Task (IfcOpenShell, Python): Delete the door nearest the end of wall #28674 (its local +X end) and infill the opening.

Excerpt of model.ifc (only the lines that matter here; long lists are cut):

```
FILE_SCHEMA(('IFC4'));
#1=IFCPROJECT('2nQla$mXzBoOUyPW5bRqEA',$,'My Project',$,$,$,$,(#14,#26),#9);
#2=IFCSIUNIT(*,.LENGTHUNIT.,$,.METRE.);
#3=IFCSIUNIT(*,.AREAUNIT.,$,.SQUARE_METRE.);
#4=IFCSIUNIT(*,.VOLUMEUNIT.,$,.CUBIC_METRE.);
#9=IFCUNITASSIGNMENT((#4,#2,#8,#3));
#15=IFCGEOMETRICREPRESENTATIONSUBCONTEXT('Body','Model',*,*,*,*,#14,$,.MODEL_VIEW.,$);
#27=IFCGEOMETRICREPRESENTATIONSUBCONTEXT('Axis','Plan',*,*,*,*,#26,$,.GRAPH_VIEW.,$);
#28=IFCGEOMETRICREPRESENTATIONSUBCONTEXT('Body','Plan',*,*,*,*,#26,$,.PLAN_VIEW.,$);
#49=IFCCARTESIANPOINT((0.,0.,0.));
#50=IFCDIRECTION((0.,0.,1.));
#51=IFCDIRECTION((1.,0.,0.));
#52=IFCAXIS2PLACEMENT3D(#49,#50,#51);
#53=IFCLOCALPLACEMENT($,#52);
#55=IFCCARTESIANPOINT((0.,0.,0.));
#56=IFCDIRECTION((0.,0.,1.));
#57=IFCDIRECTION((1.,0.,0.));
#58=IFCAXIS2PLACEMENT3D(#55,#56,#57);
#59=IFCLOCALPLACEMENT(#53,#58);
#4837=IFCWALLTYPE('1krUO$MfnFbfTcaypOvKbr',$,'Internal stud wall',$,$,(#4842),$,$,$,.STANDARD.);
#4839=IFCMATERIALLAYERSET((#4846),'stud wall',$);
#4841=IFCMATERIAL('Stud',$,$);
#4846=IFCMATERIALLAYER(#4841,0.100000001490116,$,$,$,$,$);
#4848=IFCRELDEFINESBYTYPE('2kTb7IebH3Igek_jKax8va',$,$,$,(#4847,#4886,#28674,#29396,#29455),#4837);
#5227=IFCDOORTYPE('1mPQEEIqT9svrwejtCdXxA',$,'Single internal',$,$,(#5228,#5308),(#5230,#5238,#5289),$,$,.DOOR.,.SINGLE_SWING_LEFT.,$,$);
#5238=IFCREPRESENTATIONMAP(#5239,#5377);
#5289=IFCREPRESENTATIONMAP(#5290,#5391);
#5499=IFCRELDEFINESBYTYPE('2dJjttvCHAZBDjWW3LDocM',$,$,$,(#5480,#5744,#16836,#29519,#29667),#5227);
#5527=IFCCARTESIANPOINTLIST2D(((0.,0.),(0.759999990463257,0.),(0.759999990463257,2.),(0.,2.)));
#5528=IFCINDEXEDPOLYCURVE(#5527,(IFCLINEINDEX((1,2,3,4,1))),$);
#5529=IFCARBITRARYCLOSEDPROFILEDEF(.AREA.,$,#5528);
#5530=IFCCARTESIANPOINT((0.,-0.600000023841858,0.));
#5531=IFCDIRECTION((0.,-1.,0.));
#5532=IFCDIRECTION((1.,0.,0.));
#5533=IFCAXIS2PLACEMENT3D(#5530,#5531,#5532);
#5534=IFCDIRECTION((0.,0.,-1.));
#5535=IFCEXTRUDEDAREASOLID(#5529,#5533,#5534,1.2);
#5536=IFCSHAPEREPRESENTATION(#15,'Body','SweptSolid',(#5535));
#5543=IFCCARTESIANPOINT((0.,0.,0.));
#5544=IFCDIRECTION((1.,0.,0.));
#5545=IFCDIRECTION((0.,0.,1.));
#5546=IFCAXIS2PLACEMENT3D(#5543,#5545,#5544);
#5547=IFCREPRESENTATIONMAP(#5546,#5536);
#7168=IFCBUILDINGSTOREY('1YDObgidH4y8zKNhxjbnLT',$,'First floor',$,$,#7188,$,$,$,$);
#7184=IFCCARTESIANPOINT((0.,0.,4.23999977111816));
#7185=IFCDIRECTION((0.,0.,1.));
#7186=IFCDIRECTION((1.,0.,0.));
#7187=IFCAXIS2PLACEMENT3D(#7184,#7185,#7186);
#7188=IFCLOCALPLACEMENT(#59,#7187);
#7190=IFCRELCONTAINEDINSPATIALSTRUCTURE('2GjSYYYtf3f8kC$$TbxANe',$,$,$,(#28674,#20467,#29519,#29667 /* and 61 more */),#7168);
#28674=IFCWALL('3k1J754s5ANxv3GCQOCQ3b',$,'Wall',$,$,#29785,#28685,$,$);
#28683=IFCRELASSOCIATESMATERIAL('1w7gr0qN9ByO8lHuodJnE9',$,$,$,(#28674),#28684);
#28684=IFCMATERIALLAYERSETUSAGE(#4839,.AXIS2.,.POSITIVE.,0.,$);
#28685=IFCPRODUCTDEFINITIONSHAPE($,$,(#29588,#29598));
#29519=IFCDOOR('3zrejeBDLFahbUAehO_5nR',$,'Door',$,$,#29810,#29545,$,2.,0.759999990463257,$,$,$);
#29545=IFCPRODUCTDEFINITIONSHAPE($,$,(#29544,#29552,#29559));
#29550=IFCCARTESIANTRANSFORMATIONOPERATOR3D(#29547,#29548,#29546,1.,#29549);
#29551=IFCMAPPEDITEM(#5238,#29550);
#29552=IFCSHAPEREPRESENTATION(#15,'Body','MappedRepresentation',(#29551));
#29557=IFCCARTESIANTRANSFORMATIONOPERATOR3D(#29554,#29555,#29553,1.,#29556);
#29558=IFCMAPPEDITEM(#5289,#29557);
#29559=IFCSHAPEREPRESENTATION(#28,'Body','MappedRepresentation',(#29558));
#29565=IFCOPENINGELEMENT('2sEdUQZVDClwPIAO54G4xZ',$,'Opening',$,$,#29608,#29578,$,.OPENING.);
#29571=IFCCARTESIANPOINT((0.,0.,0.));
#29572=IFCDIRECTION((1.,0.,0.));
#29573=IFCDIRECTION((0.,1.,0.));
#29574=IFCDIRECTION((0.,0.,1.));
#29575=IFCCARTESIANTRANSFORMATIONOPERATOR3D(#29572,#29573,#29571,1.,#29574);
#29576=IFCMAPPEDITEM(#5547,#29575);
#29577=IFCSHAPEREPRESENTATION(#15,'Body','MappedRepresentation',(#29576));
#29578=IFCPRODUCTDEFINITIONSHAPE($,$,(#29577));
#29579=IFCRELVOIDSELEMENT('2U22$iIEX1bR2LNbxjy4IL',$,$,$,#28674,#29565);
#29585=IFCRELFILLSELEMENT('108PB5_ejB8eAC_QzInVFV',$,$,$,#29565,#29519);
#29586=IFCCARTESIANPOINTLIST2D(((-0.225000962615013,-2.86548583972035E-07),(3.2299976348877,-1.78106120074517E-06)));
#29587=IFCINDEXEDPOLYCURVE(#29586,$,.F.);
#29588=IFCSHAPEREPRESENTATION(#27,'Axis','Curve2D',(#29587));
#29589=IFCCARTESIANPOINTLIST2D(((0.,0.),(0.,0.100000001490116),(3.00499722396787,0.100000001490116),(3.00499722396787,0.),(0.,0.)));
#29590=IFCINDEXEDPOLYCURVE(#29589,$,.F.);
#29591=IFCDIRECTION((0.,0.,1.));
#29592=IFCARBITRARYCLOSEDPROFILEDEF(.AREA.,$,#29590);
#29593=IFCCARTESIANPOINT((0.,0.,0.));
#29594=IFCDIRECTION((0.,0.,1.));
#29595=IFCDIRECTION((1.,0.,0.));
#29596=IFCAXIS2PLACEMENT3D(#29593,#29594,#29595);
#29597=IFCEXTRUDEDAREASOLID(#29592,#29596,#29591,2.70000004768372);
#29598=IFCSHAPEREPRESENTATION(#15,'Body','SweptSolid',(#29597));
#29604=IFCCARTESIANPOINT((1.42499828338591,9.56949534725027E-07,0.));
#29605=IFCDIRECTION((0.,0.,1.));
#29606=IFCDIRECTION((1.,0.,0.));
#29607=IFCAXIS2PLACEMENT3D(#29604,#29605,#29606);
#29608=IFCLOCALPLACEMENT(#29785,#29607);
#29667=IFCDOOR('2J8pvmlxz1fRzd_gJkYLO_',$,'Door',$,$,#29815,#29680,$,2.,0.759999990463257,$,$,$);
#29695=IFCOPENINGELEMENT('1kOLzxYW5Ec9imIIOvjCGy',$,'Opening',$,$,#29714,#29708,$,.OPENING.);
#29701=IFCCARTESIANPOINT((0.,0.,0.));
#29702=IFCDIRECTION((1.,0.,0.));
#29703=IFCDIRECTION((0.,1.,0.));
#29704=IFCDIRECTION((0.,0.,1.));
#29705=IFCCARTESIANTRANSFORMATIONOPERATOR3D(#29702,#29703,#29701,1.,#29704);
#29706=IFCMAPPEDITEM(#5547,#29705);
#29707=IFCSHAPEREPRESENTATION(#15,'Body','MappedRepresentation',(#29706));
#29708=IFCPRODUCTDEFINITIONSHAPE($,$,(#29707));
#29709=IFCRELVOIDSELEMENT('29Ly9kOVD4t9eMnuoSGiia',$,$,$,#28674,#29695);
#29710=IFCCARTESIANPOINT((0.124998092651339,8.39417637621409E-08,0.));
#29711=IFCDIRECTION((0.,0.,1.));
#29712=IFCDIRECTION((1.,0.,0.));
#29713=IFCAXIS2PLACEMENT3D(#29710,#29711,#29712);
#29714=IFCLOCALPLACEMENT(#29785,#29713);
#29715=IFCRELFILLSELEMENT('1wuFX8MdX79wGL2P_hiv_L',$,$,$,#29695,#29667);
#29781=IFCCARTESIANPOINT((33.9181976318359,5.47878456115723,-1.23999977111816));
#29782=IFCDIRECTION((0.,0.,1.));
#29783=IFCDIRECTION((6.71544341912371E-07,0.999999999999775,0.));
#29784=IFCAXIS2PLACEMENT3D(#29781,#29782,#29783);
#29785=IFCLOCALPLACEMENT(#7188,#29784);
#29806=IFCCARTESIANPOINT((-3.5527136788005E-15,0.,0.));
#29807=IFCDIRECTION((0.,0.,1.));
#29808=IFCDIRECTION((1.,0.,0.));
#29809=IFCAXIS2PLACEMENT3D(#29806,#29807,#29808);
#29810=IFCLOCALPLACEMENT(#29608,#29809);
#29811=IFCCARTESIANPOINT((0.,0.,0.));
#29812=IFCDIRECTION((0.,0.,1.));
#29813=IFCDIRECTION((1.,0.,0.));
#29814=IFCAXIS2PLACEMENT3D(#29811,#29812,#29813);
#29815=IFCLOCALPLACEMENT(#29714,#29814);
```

```python
import ifcopenshell
import ifcopenshell.api.feature
import ifcopenshell.api.root
import ifcopenshell.geom
import ifcopenshell.util.shape

model = ifcopenshell.open("model.ifc")
settings = ifcopenshell.geom.settings()


def volume(element):
    """Net volume in cubic metres, openings subtracted."""
    shape = ifcopenshell.geom.create_shape(settings, element)
    return ifcopenshell.util.shape.get_volume(shape.geometry)


door = model.by_id(29519)
opening = door.FillsVoids[0].RelatingOpeningElement
wall = opening.VoidsElements[0].RelatingBuildingElement
before = volume(wall)

ifcopenshell.api.root.remove_product(model, product=door)
ifcopenshell.api.feature.remove_feature(model, feature=opening)

after = volume(wall)

print(f"wall volume {before:.3f} -> {after:.3f} m3")

model.write("model_updated.ifc")
```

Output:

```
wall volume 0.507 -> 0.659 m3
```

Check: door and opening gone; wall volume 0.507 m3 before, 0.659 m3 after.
